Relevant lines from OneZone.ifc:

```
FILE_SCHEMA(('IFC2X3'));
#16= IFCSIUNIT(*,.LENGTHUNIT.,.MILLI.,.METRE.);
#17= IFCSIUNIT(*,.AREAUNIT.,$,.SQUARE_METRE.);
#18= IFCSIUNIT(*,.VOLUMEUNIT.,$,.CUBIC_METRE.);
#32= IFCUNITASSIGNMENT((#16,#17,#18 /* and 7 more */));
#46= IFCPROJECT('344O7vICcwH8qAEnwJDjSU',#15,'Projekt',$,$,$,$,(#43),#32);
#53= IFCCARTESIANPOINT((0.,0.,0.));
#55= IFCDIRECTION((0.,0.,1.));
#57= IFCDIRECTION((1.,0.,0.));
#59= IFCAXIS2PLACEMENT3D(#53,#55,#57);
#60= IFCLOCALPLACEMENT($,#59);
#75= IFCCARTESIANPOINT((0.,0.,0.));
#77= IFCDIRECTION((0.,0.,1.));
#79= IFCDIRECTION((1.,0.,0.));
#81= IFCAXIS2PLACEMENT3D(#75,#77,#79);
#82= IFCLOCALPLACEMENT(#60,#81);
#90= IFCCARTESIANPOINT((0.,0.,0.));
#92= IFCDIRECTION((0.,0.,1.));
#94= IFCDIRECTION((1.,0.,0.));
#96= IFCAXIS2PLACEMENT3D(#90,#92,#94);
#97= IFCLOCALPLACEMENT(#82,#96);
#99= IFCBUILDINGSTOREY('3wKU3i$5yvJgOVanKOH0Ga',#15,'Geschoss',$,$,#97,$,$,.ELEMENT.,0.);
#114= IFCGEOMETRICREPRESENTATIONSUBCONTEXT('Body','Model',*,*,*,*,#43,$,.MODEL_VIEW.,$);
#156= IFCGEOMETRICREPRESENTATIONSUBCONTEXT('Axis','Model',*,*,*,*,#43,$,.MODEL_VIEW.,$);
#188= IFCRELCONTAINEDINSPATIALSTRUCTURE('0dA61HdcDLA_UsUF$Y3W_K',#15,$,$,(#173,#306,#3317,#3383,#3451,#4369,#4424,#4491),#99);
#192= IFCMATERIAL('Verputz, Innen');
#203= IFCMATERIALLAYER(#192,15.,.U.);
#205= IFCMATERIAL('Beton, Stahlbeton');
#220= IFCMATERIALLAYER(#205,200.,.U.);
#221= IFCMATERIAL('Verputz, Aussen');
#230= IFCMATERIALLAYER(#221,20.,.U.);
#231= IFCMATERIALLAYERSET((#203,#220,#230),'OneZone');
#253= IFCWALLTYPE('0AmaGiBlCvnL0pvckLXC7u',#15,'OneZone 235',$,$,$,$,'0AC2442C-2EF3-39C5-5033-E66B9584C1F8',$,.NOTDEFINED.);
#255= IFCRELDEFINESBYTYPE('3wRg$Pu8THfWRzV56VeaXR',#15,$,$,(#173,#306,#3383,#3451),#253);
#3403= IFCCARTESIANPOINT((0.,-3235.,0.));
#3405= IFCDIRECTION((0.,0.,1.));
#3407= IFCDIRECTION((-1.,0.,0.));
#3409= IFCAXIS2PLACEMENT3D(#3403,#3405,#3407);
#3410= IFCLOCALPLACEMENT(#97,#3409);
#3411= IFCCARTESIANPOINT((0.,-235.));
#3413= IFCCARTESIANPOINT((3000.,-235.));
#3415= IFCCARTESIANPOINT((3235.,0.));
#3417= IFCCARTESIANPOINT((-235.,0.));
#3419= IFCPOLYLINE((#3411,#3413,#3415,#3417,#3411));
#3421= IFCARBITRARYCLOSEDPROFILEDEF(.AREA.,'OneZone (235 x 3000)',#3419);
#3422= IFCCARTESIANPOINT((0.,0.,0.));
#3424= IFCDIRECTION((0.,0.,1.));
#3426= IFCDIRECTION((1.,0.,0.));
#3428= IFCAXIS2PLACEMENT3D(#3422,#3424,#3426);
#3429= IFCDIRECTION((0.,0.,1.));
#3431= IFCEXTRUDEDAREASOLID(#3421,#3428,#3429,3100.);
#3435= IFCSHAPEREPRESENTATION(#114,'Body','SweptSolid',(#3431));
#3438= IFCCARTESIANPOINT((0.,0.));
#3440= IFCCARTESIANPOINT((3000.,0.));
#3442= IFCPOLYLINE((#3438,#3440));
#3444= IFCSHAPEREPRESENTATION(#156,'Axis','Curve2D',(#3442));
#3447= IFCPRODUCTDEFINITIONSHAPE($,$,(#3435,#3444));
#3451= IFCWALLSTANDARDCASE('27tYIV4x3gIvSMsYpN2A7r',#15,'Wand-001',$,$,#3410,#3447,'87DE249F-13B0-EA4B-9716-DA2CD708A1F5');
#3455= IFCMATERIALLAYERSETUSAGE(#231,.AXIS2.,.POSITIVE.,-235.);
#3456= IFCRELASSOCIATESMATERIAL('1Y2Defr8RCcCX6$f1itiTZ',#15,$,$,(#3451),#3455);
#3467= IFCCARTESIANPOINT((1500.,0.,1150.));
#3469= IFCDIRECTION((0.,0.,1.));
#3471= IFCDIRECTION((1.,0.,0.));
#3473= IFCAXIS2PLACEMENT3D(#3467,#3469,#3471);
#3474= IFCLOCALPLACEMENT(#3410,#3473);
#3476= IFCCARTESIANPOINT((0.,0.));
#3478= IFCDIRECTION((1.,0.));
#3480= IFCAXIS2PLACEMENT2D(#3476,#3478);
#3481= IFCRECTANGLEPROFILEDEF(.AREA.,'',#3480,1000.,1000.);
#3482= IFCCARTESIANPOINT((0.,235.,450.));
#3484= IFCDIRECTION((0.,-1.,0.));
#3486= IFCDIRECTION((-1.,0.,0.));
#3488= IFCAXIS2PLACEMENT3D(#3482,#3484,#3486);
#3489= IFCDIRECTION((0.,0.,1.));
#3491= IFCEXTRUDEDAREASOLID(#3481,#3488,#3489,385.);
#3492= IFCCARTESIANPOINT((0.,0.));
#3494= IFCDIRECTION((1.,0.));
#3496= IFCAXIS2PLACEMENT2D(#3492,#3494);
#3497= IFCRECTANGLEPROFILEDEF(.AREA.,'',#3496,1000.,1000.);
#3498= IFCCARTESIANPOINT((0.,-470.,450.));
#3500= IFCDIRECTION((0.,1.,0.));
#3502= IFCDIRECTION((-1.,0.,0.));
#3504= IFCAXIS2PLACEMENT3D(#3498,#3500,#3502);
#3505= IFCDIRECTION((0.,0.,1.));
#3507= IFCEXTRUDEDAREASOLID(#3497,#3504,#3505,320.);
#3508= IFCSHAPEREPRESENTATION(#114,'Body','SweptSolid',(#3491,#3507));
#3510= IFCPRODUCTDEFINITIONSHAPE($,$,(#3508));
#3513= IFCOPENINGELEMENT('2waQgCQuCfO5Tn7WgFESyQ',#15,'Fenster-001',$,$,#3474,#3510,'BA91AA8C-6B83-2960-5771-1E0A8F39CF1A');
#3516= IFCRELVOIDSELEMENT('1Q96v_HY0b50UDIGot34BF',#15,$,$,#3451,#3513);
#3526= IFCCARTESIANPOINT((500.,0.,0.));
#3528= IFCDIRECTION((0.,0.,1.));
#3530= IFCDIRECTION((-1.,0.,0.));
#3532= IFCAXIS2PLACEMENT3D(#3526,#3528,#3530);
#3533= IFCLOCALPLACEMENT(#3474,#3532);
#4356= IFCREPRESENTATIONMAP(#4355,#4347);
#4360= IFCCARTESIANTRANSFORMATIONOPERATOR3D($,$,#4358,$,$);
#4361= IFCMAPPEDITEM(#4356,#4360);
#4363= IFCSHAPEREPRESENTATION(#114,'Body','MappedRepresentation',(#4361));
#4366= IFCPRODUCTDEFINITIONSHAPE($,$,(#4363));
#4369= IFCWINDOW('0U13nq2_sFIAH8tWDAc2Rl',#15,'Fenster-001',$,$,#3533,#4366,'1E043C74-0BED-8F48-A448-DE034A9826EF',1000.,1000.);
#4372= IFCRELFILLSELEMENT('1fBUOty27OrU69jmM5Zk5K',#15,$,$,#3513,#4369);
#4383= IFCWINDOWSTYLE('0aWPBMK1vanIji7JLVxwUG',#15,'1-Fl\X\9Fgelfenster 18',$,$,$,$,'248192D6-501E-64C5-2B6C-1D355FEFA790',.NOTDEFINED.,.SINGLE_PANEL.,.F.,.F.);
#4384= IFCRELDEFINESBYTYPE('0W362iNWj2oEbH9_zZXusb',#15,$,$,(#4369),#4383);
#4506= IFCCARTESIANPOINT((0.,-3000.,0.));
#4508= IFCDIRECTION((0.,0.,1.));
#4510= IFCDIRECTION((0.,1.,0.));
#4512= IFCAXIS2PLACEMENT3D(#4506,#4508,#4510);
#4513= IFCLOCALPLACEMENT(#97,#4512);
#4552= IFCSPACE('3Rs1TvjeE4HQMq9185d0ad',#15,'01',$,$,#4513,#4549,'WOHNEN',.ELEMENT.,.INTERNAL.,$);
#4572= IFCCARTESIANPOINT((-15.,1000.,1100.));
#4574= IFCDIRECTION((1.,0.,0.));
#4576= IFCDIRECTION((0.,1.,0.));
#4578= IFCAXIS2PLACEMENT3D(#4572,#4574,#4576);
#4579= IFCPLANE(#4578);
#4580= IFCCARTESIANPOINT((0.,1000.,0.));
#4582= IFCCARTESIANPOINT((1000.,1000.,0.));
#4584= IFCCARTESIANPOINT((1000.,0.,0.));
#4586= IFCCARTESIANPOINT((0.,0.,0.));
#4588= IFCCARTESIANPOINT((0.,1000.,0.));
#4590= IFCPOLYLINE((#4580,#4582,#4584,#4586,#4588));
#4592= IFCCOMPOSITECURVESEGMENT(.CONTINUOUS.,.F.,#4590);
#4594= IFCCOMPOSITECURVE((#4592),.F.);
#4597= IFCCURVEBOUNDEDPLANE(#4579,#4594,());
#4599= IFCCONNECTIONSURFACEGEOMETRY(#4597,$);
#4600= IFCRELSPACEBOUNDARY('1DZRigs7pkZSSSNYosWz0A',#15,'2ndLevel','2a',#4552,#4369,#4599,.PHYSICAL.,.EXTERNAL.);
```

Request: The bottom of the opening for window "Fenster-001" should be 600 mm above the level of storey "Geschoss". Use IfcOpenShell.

```python
import numpy as np
import ifcopenshell
import ifcopenshell.api.geometry
import ifcopenshell.geom
import ifcopenshell.util.element
import ifcopenshell.util.placement
import ifcopenshell.util.shape
import ifcopenshell.util.unit

model = ifcopenshell.open("OneZone.ifc")
unit_scale = ifcopenshell.util.unit.calculate_unit_scale(model)

window = model.by_guid("0U13nq2_sFIAH8tWDAc2Rl")
opening = window.FillsVoids[0].RelatingOpeningElement
storey = ifcopenshell.util.element.get_container(window, ifc_class="IfcBuildingStorey")
level = ifcopenshell.util.placement.get_local_placement(storey.ObjectPlacement)[2, 3]

# The opening's origin need not be at the sill, so measure its lowest point.
shape = ifcopenshell.geom.create_shape(ifcopenshell.geom.settings(), opening)
bottom = ifcopenshell.util.shape.get_shape_bottom_elevation(shape, shape.geometry) / unit_scale
dz = level + 600.0 - bottom

shift = np.array([0.0, 0.0, dz])
# The window is placed relative to its opening, so it follows when the opening moves.
matrix = ifcopenshell.util.placement.get_local_placement(opening.ObjectPlacement)
matrix[:3, 3] += shift
ifcopenshell.api.geometry.edit_object_placement(
    model, product=opening, matrix=matrix, is_si=False, should_transform_children=True
)

# Space boundary surfaces are stored in each space's coordinates; move them too.
for rel in window.ProvidesBoundaries:
    if not rel.ConnectionGeometry:
        continue
    surface = rel.ConnectionGeometry.SurfaceOnRelatingElement.BasisSurface
    space_matrix = ifcopenshell.util.placement.get_local_placement(rel.RelatingSpace.ObjectPlacement)
    point = np.array(surface.Position.Location.Coordinates) + space_matrix[:3, :3].T @ shift
    surface.Position = model.createIfcAxis2Placement3D(
        model.createIfcCartesianPoint(point.tolist()), surface.Position.Axis, surface.Position.RefDirection
    )

print(f"moved by {dz * unit_scale:+.3f} m")

model.write("OneZone_edited.ifc")
```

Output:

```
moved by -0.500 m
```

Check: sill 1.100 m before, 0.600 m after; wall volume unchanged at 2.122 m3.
